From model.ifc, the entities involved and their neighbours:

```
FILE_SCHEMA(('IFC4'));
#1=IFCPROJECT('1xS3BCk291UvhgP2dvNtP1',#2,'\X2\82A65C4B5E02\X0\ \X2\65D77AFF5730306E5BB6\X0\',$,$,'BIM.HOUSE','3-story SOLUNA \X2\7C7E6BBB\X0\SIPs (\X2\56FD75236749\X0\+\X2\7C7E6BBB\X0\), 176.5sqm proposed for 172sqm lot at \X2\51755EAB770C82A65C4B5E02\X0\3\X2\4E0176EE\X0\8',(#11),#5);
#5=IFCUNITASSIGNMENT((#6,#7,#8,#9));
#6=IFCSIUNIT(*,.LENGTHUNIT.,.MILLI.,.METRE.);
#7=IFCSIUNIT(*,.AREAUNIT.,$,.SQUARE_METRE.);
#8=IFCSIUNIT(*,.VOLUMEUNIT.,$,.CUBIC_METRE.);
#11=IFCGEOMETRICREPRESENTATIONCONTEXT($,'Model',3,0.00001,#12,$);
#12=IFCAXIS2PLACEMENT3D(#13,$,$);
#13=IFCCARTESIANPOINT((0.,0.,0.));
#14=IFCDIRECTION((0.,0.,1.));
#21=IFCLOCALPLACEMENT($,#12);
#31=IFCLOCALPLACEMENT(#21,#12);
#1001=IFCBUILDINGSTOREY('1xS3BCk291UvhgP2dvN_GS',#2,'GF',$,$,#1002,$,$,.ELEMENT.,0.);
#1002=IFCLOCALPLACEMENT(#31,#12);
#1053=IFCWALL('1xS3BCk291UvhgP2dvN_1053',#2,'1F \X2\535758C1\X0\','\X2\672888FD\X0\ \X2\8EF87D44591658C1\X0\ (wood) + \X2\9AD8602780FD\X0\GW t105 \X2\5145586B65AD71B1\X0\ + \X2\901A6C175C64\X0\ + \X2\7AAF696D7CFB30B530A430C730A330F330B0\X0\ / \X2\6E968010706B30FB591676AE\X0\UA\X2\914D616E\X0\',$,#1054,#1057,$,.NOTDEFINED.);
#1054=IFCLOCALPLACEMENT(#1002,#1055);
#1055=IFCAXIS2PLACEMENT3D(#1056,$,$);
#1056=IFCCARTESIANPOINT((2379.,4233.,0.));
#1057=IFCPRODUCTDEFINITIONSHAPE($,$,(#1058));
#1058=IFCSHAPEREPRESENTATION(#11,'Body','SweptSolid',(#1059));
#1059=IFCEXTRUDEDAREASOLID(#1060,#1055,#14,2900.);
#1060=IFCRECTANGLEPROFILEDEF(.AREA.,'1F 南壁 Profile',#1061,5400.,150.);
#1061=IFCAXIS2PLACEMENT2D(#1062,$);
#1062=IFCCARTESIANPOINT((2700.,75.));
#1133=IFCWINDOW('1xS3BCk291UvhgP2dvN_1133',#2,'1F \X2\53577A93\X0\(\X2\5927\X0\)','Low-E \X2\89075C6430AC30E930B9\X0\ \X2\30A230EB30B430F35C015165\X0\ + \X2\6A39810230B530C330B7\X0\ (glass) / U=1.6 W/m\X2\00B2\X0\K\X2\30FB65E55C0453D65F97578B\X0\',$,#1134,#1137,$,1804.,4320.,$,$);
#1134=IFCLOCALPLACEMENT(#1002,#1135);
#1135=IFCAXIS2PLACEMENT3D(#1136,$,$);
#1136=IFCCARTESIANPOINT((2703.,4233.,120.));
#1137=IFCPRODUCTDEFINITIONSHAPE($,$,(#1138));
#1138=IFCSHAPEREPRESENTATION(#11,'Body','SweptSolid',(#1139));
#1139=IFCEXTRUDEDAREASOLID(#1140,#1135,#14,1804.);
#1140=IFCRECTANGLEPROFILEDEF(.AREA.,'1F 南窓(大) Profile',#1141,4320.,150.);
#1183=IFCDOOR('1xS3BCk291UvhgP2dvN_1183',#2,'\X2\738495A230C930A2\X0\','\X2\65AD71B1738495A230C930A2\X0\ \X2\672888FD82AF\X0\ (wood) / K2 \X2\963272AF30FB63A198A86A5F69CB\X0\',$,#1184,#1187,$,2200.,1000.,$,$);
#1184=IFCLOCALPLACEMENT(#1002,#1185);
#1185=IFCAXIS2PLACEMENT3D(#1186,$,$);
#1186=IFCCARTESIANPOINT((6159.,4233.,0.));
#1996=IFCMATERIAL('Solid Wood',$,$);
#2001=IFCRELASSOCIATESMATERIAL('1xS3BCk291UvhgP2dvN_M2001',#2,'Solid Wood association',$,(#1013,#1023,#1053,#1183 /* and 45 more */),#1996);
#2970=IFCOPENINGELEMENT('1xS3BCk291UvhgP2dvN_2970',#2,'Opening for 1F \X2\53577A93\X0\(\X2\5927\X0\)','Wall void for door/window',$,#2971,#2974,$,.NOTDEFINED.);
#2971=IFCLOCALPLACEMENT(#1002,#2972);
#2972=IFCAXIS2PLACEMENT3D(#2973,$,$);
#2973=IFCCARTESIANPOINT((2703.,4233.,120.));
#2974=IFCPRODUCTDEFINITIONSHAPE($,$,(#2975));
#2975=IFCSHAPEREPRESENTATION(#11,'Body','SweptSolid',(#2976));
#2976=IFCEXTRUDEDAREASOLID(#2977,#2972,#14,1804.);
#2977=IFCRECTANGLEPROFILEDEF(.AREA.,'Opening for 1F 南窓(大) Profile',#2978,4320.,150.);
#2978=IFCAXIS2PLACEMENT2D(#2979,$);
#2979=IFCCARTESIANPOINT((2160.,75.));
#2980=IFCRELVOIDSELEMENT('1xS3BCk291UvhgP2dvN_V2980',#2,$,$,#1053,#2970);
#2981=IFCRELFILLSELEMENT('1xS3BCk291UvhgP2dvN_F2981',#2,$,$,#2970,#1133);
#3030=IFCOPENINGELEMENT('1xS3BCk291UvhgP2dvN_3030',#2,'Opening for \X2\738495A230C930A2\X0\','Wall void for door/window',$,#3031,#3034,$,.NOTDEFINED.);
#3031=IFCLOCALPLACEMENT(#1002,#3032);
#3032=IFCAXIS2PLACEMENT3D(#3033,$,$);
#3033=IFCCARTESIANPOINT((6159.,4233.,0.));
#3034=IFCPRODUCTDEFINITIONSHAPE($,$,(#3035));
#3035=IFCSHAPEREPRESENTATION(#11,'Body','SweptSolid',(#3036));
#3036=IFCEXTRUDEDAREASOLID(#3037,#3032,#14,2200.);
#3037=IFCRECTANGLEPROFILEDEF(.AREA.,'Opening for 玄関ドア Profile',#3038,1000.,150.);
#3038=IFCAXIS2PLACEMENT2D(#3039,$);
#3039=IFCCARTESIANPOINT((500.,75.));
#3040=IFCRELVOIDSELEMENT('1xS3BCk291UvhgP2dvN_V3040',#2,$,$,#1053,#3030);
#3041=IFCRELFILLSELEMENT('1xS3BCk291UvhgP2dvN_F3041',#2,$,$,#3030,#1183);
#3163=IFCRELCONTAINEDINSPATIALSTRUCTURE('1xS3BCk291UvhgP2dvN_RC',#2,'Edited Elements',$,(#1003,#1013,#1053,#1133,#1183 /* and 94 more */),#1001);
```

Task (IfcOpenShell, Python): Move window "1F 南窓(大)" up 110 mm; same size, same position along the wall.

```python
import numpy as np
import ifcopenshell
import ifcopenshell.api.geometry
import ifcopenshell.util.placement
import ifcopenshell.util.unit

model = ifcopenshell.open("model.ifc")
unit_scale = ifcopenshell.util.unit.calculate_unit_scale(model)

window = model.by_guid("1xS3BCk291UvhgP2dvN_1133")
opening = window.FillsVoids[0].RelatingOpeningElement
dz = 110.0

shift = np.array([0.0, 0.0, dz])
# The window is not placed relative to its opening, so move both.
for product in (opening, window):
    matrix = ifcopenshell.util.placement.get_local_placement(product.ObjectPlacement)
    matrix[:3, 3] += shift
    ifcopenshell.api.geometry.edit_object_placement(model, product=product, matrix=matrix, is_si=False)

print(f"moved by {dz * unit_scale:+.3f} m")

model.write("model_v2.ifc")
```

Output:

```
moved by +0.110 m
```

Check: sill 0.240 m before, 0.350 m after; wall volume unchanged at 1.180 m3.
